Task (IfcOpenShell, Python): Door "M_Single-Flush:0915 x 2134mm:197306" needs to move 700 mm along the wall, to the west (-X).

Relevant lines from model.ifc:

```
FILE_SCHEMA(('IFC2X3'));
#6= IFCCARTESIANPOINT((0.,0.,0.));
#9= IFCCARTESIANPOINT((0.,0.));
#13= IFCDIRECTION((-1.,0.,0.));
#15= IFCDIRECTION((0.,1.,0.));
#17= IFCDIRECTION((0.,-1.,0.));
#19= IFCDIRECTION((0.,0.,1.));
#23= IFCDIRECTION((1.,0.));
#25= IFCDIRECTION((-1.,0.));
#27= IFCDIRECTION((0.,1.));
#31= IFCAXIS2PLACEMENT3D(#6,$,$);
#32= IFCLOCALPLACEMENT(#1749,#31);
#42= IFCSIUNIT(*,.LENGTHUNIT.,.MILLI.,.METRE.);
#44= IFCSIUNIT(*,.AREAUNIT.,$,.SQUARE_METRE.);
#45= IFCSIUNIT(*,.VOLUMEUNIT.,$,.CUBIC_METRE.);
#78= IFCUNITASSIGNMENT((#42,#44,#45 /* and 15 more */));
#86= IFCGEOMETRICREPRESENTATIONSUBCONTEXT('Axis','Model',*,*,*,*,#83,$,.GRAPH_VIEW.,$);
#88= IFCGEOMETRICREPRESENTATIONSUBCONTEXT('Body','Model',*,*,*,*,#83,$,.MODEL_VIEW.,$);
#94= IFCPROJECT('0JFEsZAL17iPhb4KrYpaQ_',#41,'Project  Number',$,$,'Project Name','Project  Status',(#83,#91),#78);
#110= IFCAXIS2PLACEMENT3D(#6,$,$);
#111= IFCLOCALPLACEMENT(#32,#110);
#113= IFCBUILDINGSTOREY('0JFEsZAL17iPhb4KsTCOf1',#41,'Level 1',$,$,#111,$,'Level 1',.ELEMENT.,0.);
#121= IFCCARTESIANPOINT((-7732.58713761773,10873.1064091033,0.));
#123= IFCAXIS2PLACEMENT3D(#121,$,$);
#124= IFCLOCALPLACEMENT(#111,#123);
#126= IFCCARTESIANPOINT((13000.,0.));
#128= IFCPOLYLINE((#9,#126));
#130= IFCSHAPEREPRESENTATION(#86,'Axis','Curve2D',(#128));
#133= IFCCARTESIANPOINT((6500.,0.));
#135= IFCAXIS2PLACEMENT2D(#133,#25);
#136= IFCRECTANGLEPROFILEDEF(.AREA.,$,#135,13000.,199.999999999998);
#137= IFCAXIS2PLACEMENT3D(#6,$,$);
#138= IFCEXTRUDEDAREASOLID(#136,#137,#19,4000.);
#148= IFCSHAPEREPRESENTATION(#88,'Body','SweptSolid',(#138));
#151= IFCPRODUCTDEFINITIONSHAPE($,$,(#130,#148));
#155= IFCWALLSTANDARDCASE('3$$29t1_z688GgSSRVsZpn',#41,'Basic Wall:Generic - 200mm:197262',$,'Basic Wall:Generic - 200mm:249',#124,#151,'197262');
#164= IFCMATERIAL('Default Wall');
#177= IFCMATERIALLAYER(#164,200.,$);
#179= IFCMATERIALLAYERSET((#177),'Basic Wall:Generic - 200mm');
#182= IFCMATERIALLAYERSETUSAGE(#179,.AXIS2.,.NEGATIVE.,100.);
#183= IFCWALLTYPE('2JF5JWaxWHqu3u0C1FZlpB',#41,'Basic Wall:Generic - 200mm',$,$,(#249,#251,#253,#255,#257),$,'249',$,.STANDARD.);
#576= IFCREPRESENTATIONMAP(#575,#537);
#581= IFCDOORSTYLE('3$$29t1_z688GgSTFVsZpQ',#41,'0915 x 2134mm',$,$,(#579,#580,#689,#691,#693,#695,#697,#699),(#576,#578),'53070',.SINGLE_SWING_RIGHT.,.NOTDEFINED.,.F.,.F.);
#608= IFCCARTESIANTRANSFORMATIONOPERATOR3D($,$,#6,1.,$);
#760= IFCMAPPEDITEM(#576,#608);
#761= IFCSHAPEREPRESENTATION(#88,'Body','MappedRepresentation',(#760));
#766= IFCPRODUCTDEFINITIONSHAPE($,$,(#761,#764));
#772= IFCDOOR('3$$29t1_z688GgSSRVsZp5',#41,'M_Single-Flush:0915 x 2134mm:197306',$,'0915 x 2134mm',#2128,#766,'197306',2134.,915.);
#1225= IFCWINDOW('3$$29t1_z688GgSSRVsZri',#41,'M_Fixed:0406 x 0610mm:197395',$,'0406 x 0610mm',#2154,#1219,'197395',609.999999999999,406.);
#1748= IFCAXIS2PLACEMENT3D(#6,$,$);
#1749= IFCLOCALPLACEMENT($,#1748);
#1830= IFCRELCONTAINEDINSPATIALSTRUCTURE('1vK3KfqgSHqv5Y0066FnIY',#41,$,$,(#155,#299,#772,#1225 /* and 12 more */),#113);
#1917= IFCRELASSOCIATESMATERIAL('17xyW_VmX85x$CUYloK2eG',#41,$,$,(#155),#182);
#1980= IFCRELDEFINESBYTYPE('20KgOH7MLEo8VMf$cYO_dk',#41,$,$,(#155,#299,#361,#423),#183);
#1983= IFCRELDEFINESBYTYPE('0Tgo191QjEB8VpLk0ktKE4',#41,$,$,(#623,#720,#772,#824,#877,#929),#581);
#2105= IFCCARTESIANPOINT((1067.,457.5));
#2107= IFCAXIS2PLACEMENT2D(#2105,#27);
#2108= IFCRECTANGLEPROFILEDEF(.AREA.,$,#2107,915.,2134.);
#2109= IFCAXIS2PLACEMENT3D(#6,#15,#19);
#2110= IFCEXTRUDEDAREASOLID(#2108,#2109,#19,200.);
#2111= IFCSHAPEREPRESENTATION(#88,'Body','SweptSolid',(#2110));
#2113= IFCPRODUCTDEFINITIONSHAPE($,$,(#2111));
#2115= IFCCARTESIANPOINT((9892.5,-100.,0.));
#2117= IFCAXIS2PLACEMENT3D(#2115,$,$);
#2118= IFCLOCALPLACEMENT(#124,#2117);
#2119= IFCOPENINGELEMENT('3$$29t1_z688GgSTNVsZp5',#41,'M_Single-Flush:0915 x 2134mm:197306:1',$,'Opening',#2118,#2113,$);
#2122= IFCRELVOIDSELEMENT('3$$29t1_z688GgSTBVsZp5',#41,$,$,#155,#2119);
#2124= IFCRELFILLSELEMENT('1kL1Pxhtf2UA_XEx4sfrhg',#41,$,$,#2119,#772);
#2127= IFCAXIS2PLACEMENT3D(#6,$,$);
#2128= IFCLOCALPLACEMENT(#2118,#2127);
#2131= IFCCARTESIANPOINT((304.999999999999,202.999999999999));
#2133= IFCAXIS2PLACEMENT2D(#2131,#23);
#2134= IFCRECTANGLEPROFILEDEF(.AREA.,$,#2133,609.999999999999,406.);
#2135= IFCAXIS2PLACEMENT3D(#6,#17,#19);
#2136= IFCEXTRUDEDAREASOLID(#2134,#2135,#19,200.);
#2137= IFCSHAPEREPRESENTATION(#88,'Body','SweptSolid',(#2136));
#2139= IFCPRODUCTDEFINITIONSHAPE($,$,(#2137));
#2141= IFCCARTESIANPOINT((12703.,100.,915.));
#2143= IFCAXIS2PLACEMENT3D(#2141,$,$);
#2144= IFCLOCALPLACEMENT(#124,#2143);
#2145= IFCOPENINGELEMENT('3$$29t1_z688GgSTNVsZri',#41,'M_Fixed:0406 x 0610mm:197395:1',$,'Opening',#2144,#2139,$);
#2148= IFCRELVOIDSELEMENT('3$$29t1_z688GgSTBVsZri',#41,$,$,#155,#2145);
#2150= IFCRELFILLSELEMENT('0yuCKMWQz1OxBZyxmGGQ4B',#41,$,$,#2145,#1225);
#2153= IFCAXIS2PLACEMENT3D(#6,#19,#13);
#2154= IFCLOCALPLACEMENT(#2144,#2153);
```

```python
import ifcopenshell
import ifcopenshell.api.geometry
import ifcopenshell.util.placement
import ifcopenshell.util.unit

model = ifcopenshell.open("model.ifc")
unit_scale = ifcopenshell.util.unit.calculate_unit_scale(model)

door = model.by_guid("3$$29t1_z688GgSSRVsZp5")
opening = door.FillsVoids[0].RelatingOpeningElement
wall = opening.VoidsElements[0].RelatingBuildingElement

wall_matrix = ifcopenshell.util.placement.get_local_placement(wall.ObjectPlacement)
shift = wall_matrix[:3, 0] * -0.7 / unit_scale
before = ifcopenshell.util.placement.get_local_placement(door.ObjectPlacement)[:3, 3].copy()

# The door is placed relative to its opening, so it follows when the opening moves.
matrix = ifcopenshell.util.placement.get_local_placement(opening.ObjectPlacement)
matrix[:3, 3] += shift
ifcopenshell.api.geometry.edit_object_placement(
    model, product=opening, matrix=matrix, is_si=False, should_transform_children=True
)

after = ifcopenshell.util.placement.get_local_placement(door.ObjectPlacement)[:3, 3]
print("door moved by", (after - before).round(3) + 0.0)

model.write("model_updated.ifc")
```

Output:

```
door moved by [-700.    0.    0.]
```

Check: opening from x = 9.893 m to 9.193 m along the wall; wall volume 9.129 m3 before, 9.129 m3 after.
